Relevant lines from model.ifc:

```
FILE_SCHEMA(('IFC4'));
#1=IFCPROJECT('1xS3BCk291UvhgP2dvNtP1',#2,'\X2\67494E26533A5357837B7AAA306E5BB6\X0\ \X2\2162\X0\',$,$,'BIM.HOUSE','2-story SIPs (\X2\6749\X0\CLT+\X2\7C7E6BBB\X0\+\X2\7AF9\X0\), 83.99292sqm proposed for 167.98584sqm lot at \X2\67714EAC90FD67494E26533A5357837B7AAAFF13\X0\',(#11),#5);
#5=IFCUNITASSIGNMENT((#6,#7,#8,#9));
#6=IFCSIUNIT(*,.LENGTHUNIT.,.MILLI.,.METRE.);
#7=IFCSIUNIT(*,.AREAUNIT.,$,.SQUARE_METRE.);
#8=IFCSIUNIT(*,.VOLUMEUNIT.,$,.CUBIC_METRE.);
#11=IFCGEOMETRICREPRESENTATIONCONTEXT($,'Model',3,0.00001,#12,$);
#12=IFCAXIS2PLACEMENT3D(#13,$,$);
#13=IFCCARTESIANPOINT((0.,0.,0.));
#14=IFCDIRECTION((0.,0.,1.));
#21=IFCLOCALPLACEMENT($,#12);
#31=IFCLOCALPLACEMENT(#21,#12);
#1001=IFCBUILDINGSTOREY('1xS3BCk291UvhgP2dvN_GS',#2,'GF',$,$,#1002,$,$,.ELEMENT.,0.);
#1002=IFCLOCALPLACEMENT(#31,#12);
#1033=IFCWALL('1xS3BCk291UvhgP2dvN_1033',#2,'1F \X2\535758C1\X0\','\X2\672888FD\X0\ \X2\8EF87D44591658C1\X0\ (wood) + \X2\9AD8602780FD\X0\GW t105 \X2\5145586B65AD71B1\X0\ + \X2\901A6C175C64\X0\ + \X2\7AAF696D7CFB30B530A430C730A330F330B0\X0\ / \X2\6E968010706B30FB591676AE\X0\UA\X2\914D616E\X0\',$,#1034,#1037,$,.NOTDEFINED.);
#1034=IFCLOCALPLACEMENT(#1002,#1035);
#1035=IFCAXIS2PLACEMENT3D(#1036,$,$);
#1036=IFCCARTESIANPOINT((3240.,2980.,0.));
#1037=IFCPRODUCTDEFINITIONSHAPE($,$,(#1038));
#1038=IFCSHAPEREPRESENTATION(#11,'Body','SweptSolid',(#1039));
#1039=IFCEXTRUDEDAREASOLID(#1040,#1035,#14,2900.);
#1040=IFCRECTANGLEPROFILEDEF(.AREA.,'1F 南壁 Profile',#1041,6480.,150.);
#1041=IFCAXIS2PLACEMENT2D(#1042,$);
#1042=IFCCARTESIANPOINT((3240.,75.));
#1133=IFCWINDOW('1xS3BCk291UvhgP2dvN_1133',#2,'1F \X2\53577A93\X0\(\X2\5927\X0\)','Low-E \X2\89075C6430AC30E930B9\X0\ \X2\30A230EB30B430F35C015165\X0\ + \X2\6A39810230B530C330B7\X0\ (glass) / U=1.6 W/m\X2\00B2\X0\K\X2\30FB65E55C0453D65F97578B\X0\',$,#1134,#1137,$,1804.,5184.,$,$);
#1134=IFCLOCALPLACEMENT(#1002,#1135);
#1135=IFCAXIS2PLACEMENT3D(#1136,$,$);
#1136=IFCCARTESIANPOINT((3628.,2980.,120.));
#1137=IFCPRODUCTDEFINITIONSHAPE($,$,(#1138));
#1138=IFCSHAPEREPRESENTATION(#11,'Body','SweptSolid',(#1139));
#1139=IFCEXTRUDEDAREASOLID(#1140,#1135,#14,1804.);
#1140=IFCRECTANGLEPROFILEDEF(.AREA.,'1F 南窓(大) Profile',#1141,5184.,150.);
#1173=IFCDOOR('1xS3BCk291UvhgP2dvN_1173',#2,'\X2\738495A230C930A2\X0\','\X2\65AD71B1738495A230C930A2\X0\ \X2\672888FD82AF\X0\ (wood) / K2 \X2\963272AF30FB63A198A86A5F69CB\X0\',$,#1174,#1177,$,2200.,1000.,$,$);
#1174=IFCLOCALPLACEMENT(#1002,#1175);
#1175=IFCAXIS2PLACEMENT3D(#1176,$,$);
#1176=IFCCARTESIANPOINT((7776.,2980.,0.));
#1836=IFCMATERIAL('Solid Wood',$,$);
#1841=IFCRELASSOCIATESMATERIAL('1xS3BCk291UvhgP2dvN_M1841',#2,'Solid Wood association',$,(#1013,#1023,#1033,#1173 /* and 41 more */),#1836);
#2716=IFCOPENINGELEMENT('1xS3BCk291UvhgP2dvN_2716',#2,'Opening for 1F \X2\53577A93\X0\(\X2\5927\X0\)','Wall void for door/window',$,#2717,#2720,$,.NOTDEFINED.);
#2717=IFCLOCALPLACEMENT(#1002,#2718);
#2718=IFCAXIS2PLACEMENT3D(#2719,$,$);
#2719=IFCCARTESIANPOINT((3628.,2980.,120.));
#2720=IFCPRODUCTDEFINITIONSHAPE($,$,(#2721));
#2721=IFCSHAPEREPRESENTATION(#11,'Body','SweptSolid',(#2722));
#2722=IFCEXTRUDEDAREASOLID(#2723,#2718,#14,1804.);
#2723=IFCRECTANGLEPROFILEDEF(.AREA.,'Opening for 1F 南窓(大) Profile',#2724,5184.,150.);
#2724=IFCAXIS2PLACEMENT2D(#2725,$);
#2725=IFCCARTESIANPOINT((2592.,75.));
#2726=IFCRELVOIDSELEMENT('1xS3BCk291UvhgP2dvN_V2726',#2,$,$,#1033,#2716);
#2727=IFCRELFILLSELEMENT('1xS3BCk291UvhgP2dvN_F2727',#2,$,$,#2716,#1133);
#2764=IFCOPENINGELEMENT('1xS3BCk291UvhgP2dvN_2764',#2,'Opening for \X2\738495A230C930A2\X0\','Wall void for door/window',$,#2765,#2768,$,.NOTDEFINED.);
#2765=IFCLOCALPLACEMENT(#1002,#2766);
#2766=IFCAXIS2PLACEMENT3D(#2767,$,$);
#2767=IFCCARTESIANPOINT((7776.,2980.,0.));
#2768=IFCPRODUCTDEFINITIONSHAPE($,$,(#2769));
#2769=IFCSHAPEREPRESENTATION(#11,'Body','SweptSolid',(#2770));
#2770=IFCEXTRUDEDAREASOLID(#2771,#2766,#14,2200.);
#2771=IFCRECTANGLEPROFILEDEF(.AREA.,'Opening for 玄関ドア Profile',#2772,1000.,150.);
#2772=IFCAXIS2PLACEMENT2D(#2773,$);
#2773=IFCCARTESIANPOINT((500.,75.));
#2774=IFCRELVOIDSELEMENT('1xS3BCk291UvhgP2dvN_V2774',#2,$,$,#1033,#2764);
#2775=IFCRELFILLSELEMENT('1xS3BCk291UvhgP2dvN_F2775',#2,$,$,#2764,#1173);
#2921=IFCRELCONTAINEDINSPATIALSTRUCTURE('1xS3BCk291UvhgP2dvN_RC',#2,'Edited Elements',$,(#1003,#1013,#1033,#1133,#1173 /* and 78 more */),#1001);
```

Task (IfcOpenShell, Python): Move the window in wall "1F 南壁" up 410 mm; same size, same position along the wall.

```python
import numpy as np
import ifcopenshell
import ifcopenshell.api.geometry
import ifcopenshell.util.placement
import ifcopenshell.util.unit

model = ifcopenshell.open("model.ifc")
unit_scale = ifcopenshell.util.unit.calculate_unit_scale(model)

window = model.by_guid("1xS3BCk291UvhgP2dvN_1133")
opening = window.FillsVoids[0].RelatingOpeningElement
dz = 0.41 / unit_scale

shift = np.array([0.0, 0.0, dz])
# The window is not placed relative to its opening, so move both.
for product in (opening, window):
    matrix = ifcopenshell.util.placement.get_local_placement(product.ObjectPlacement)
    matrix[:3, 3] += shift
    ifcopenshell.api.geometry.edit_object_placement(model, product=product, matrix=matrix, is_si=False)

print(f"moved by {dz * unit_scale:+.3f} m")

model.write("model-out.ifc")
```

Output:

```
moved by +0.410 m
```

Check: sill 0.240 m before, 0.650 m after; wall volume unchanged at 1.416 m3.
